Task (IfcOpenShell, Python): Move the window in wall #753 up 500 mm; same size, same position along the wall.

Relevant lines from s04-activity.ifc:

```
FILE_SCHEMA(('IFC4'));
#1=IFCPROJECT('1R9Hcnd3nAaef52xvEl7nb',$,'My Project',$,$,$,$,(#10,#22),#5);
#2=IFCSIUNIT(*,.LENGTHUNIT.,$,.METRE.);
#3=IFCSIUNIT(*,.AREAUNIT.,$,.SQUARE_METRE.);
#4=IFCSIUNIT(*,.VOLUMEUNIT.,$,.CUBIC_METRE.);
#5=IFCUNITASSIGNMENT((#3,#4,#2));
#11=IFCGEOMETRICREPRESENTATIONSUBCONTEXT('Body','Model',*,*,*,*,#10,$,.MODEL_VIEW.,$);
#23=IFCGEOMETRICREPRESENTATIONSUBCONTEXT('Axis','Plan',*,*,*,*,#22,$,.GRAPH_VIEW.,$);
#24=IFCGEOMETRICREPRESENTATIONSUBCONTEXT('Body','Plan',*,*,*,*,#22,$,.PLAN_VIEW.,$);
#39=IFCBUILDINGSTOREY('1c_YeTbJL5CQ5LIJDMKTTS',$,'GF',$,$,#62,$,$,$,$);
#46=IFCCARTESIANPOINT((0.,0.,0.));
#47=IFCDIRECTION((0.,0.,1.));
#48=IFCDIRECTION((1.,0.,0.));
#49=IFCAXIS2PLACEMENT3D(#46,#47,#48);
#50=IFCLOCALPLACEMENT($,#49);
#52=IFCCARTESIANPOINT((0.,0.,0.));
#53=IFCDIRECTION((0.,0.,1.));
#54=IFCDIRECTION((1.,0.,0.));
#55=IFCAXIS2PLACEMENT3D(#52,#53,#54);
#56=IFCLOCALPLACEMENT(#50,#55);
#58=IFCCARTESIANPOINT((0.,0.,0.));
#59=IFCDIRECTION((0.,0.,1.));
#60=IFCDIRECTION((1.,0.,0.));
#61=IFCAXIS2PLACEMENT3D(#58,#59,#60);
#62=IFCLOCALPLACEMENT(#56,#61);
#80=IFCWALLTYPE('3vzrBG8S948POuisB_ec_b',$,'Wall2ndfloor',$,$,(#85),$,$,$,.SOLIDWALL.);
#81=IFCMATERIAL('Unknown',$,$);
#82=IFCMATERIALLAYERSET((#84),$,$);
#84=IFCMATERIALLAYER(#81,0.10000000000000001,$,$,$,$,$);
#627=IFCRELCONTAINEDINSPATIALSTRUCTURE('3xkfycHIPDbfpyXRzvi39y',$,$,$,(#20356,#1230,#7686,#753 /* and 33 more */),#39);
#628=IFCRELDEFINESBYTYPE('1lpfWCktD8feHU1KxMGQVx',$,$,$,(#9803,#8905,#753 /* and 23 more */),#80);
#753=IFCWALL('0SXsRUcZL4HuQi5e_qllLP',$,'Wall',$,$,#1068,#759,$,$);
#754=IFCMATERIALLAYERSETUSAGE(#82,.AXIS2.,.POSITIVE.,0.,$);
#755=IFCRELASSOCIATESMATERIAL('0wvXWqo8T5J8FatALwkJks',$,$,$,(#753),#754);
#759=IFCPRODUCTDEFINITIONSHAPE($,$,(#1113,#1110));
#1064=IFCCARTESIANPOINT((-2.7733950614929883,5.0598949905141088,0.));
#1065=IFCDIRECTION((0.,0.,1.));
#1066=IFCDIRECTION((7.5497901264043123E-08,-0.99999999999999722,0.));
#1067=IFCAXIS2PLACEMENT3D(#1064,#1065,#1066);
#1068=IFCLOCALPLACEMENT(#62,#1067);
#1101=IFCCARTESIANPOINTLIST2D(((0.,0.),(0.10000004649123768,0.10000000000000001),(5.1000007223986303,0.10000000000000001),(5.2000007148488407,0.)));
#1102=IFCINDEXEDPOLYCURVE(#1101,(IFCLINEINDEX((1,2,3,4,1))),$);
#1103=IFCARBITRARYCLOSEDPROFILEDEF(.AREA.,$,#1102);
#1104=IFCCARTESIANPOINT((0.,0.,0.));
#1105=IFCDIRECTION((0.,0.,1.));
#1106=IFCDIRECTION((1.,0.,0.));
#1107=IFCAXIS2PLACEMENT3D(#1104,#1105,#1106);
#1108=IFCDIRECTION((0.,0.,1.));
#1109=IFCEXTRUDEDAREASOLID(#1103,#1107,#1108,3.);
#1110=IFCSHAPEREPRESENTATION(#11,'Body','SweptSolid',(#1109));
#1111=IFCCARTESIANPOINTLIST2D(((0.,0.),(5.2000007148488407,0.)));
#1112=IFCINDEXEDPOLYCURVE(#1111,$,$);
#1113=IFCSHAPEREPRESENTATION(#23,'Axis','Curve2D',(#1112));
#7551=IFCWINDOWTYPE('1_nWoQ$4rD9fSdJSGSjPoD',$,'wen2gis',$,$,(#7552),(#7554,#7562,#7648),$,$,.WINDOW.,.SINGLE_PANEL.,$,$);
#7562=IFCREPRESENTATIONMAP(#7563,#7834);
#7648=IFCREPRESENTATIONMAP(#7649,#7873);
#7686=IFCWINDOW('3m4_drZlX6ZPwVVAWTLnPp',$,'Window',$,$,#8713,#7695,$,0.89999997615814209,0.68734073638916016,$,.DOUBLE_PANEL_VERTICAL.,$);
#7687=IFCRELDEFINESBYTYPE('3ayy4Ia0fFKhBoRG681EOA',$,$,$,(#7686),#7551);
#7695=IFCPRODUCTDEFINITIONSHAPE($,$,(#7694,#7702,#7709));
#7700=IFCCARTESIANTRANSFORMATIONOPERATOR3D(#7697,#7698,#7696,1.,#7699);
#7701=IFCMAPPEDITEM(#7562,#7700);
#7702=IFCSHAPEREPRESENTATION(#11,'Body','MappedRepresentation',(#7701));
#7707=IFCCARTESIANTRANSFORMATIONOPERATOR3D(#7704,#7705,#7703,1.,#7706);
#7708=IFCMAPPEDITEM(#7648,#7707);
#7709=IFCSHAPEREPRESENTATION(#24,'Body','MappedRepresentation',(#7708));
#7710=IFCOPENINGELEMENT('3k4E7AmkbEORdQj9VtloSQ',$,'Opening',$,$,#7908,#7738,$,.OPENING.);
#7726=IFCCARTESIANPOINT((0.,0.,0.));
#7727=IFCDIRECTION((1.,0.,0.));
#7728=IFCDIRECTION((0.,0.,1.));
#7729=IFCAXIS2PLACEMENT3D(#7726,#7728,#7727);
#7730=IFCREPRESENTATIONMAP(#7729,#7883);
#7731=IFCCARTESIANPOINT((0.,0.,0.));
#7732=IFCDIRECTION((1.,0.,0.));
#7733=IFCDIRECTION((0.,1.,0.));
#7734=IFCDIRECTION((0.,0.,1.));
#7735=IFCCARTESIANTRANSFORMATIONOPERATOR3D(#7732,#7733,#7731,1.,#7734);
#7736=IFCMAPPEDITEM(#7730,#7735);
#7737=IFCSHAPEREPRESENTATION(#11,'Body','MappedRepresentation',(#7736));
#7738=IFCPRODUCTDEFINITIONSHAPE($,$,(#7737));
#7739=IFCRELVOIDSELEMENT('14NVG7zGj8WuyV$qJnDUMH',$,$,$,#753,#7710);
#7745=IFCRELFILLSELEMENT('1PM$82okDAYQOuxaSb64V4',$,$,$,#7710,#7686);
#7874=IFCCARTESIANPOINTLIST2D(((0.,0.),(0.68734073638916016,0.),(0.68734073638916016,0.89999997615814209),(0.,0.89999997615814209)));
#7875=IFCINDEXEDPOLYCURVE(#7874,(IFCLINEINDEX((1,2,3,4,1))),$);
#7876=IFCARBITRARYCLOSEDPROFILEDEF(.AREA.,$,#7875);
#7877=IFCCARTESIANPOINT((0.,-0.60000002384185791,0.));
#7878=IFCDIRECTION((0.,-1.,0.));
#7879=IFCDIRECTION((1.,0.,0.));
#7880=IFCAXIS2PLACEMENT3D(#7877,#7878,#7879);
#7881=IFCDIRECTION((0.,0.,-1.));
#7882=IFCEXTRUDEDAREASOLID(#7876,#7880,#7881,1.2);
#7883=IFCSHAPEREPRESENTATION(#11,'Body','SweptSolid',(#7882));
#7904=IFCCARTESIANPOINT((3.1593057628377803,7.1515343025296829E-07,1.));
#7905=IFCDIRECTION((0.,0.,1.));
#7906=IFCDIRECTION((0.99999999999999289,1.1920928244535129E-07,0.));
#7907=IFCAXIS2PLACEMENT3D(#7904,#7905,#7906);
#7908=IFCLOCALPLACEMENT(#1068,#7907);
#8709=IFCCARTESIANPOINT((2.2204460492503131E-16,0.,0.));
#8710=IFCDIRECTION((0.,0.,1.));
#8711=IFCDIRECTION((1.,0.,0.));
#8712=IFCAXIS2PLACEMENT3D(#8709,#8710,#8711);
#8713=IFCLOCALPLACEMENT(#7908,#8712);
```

```python
import numpy as np
import ifcopenshell
import ifcopenshell.api.geometry
import ifcopenshell.util.placement
import ifcopenshell.util.unit

model = ifcopenshell.open("s04-activity.ifc")
unit_scale = ifcopenshell.util.unit.calculate_unit_scale(model)

window = model.by_guid("3m4_drZlX6ZPwVVAWTLnPp")
opening = window.FillsVoids[0].RelatingOpeningElement
dz = 0.5

shift = np.array([0.0, 0.0, dz])
# The window is placed relative to its opening, so it follows when the opening moves.
matrix = ifcopenshell.util.placement.get_local_placement(opening.ObjectPlacement)
matrix[:3, 3] += shift
ifcopenshell.api.geometry.edit_object_placement(
    model, product=opening, matrix=matrix, is_si=False, should_transform_children=True
)

print(f"moved by {dz * unit_scale:+.3f} m")

model.write("s04-activity_edited.ifc")
```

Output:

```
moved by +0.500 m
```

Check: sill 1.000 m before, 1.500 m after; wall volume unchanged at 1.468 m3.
